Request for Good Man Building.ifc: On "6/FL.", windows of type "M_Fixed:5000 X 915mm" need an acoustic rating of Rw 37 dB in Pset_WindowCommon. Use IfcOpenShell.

First a look at what the model holds.

```python
import ifcopenshell
import ifcopenshell.util.element

model = ifcopenshell.open("Good Man Building.ifc")
print(model.schema)
storey = next(s for s in model.by_type("IfcBuildingStorey") if s.Name == "6/FL.")
windows = [e for e in ifcopenshell.util.element.get_decomposition(storey) if e.is_a("IfcWindow")]
seen = {}
for e in windows:
    element_type = ifcopenshell.util.element.get_type(e)
    key = (element_type.Name if element_type != e and element_type else None, ifcopenshell.util.element.get_pset(e, "Pset_WindowCommon", "AcousticRating"))
    seen[key] = seen.get(key, 0) + 1
for (name, value), count in sorted(seen.items(), key=str):
    print(count, "x", name, "|", value)
```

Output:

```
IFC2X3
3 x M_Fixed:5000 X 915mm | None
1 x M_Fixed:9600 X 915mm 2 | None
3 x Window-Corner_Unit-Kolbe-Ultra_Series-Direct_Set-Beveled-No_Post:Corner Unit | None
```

```python
import ifcopenshell
import ifcopenshell.api.pset
import ifcopenshell.util.element

model = ifcopenshell.open("Good Man Building.ifc")

storey = next(s for s in model.by_type("IfcBuildingStorey") if s.Name == "6/FL.")
windows = [e for e in ifcopenshell.util.element.get_decomposition(storey) if e.is_a("IfcWindow")]

count = 0
for e in windows:
    element_type = ifcopenshell.util.element.get_type(e)
    if element_type in (None, e) or element_type.Name != "M_Fixed:5000 X 915mm":
        continue
    # add_pset returns the element's existing set when there is one.
    pset = ifcopenshell.api.pset.add_pset(model, product=e, name="Pset_WindowCommon")
    ifcopenshell.api.pset.edit_pset(model, pset=pset, properties={"AcousticRating": "Rw 37 dB"})
    count += 1

print(count, "windows updated")

model.write("Good Man Building_v2.ifc")
```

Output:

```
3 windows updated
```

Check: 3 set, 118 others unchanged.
